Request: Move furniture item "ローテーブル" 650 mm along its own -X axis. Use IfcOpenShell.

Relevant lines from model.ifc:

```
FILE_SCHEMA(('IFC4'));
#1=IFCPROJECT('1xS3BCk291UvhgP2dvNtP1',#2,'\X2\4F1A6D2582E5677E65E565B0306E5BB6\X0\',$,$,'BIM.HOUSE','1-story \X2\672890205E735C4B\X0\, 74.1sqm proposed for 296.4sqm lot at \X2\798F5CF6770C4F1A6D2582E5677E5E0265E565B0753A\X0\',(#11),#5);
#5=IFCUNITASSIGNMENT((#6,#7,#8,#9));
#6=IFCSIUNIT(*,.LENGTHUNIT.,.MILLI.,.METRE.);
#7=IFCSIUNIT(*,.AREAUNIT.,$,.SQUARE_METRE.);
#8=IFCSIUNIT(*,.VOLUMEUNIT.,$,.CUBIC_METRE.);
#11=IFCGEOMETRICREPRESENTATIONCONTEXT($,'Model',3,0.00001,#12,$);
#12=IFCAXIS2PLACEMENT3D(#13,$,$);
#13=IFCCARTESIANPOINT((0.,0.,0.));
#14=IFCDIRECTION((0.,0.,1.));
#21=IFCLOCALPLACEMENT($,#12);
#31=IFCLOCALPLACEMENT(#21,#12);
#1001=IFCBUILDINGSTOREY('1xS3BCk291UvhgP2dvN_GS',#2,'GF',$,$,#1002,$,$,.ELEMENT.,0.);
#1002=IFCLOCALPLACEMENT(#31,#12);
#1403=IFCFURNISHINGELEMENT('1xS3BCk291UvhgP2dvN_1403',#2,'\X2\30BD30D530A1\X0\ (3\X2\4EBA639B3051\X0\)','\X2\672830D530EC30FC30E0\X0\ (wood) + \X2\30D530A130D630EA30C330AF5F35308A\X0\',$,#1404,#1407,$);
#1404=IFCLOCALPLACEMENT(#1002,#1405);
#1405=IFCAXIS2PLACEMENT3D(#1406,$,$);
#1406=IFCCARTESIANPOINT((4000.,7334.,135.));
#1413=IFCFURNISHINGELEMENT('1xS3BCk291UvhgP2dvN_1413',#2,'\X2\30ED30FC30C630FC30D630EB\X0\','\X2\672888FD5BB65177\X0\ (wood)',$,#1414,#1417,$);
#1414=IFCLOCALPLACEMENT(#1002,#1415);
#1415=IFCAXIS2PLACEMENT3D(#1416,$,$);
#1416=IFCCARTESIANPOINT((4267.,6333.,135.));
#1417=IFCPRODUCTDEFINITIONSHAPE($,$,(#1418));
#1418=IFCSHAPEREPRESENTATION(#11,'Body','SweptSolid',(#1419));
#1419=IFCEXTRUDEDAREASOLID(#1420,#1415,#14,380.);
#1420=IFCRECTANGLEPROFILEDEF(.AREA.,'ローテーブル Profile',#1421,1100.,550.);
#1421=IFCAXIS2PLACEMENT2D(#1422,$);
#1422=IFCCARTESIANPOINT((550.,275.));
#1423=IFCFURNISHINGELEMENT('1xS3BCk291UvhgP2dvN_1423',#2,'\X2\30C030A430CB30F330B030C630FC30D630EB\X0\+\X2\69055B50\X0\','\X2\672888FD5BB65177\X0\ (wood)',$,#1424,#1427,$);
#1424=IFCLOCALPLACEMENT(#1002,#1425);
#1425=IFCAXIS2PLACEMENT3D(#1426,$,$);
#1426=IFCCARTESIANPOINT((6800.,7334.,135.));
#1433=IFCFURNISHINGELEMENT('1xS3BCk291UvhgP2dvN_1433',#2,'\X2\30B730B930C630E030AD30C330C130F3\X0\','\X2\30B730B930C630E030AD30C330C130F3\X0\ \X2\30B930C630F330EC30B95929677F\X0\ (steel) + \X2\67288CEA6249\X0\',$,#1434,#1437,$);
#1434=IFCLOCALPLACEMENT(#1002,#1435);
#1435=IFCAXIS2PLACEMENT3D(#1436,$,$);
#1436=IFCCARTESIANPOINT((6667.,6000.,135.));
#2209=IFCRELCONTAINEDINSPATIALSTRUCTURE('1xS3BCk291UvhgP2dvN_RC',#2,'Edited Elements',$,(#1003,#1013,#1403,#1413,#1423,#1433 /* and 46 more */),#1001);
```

```python
import ifcopenshell
import ifcopenshell.api.geometry
import ifcopenshell.util.placement

model = ifcopenshell.open("model.ifc")

item = model.by_guid("1xS3BCk291UvhgP2dvN_1413")
matrix = ifcopenshell.util.placement.get_local_placement(item.ObjectPlacement)
matrix[:3, 3] -= matrix[:3, 0] * 650.0
ifcopenshell.api.geometry.edit_object_placement(model, product=item, matrix=matrix, is_si=False)

print(ifcopenshell.util.placement.get_local_placement(item.ObjectPlacement).round(3) + 0.0)

model.write("model_v2.ifc")
```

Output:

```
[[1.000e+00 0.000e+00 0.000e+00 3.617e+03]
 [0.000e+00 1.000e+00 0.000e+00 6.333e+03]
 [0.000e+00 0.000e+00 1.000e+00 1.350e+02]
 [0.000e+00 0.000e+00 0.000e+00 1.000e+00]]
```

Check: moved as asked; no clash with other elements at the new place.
